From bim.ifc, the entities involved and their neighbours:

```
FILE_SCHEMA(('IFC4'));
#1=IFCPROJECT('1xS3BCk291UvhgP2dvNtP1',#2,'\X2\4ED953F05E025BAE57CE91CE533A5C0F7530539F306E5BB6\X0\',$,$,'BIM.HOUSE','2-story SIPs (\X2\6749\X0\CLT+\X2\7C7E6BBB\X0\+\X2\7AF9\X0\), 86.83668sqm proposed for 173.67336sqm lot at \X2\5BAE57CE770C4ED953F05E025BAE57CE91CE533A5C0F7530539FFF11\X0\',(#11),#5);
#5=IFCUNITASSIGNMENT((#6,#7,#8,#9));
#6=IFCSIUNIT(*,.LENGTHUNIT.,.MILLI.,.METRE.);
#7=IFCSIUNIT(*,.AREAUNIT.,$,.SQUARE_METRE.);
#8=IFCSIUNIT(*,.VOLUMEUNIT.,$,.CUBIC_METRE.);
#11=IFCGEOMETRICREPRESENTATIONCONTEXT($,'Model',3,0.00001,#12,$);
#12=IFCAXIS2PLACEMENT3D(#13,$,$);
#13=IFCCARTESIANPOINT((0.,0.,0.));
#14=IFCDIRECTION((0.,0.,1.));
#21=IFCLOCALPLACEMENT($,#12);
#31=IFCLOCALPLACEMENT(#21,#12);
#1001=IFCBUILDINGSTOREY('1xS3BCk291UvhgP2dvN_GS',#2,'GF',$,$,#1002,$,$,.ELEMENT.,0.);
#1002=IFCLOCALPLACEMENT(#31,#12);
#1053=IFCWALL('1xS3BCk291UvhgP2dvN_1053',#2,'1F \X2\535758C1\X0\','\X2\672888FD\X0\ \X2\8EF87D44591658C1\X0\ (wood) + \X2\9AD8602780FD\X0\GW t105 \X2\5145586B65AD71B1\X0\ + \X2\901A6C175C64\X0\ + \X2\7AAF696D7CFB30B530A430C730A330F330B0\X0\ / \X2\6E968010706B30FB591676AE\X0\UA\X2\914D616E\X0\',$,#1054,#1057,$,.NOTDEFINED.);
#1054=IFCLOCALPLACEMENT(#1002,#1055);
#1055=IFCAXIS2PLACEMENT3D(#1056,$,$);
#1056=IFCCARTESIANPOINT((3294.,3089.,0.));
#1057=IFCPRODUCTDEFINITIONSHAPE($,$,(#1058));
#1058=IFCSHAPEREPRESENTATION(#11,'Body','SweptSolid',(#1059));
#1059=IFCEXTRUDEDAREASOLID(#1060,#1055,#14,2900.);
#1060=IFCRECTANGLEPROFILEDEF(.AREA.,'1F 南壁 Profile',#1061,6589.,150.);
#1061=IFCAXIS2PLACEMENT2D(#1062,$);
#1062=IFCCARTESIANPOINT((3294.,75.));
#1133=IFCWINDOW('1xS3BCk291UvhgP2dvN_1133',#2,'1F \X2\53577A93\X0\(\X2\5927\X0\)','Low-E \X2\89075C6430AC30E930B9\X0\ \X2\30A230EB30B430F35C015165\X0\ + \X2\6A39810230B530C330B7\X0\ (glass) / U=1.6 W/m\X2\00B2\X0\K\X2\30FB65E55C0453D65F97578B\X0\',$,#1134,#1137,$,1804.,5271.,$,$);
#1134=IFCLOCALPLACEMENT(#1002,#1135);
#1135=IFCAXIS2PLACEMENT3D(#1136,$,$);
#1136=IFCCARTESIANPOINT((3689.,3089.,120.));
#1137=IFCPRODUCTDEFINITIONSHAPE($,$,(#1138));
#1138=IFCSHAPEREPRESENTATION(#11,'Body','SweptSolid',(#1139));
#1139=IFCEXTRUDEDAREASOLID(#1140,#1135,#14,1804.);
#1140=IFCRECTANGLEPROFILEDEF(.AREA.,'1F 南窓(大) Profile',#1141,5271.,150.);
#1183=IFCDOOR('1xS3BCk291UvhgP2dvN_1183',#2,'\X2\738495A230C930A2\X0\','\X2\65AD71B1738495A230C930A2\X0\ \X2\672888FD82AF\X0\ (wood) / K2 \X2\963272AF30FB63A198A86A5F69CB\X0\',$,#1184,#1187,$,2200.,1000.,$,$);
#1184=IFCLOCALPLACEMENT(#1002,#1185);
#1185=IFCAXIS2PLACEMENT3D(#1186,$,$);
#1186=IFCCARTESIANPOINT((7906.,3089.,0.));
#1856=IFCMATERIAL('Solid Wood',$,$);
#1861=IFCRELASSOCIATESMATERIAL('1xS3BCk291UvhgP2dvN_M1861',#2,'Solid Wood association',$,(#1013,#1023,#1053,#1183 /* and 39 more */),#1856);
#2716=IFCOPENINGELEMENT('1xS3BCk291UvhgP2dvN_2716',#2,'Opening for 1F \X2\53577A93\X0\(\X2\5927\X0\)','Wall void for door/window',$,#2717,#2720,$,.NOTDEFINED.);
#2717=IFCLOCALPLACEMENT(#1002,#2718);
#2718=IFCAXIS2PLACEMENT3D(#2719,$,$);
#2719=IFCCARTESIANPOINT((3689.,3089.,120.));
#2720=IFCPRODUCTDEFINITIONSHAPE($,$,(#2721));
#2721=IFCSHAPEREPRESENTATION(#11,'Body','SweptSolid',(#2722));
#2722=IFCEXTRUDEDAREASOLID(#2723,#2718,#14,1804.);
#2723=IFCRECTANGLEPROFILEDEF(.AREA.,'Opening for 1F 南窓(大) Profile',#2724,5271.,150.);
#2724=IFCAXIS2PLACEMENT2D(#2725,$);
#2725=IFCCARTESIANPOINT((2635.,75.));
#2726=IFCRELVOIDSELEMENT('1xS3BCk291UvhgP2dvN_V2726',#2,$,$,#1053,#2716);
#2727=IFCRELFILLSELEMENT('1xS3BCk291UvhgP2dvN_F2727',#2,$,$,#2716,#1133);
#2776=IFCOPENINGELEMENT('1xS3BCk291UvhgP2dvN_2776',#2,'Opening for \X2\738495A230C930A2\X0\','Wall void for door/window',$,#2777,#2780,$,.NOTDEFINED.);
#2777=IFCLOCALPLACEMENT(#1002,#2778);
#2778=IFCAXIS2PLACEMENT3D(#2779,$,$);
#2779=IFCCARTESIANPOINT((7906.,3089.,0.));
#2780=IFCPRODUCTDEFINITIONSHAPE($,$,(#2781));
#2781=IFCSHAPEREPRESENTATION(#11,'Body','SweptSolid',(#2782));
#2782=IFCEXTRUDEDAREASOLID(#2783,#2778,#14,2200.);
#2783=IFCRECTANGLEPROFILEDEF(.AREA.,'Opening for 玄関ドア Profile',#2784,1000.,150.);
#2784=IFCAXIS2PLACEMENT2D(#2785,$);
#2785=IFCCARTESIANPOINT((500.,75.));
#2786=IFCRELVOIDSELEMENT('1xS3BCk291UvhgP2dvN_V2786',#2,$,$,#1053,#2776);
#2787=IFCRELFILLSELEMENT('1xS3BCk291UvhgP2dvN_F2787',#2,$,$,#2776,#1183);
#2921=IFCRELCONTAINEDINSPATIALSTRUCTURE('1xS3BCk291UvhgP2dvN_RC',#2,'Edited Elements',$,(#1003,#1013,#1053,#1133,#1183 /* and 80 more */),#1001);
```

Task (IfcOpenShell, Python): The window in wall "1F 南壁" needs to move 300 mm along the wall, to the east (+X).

```python
import ifcopenshell
import ifcopenshell.api.geometry
import ifcopenshell.util.placement

model = ifcopenshell.open("bim.ifc")

window = model.by_guid("1xS3BCk291UvhgP2dvN_1133")
opening = window.FillsVoids[0].RelatingOpeningElement
wall = opening.VoidsElements[0].RelatingBuildingElement

wall_matrix = ifcopenshell.util.placement.get_local_placement(wall.ObjectPlacement)
shift = wall_matrix[:3, 0] * 300.0
before = ifcopenshell.util.placement.get_local_placement(window.ObjectPlacement)[:3, 3].copy()

# The window is not placed relative to its opening, so move both.
for product in (opening, window):
    matrix = ifcopenshell.util.placement.get_local_placement(product.ObjectPlacement)
    matrix[:3, 3] += shift
    ifcopenshell.api.geometry.edit_object_placement(model, product=product, matrix=matrix, is_si=False)

after = ifcopenshell.util.placement.get_local_placement(window.ObjectPlacement)[:3, 3]
print("window moved by", (after - before).round(3) + 0.0)

model.write("bim_v2.ifc")
```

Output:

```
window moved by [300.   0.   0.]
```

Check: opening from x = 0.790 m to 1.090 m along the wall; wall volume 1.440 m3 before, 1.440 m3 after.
